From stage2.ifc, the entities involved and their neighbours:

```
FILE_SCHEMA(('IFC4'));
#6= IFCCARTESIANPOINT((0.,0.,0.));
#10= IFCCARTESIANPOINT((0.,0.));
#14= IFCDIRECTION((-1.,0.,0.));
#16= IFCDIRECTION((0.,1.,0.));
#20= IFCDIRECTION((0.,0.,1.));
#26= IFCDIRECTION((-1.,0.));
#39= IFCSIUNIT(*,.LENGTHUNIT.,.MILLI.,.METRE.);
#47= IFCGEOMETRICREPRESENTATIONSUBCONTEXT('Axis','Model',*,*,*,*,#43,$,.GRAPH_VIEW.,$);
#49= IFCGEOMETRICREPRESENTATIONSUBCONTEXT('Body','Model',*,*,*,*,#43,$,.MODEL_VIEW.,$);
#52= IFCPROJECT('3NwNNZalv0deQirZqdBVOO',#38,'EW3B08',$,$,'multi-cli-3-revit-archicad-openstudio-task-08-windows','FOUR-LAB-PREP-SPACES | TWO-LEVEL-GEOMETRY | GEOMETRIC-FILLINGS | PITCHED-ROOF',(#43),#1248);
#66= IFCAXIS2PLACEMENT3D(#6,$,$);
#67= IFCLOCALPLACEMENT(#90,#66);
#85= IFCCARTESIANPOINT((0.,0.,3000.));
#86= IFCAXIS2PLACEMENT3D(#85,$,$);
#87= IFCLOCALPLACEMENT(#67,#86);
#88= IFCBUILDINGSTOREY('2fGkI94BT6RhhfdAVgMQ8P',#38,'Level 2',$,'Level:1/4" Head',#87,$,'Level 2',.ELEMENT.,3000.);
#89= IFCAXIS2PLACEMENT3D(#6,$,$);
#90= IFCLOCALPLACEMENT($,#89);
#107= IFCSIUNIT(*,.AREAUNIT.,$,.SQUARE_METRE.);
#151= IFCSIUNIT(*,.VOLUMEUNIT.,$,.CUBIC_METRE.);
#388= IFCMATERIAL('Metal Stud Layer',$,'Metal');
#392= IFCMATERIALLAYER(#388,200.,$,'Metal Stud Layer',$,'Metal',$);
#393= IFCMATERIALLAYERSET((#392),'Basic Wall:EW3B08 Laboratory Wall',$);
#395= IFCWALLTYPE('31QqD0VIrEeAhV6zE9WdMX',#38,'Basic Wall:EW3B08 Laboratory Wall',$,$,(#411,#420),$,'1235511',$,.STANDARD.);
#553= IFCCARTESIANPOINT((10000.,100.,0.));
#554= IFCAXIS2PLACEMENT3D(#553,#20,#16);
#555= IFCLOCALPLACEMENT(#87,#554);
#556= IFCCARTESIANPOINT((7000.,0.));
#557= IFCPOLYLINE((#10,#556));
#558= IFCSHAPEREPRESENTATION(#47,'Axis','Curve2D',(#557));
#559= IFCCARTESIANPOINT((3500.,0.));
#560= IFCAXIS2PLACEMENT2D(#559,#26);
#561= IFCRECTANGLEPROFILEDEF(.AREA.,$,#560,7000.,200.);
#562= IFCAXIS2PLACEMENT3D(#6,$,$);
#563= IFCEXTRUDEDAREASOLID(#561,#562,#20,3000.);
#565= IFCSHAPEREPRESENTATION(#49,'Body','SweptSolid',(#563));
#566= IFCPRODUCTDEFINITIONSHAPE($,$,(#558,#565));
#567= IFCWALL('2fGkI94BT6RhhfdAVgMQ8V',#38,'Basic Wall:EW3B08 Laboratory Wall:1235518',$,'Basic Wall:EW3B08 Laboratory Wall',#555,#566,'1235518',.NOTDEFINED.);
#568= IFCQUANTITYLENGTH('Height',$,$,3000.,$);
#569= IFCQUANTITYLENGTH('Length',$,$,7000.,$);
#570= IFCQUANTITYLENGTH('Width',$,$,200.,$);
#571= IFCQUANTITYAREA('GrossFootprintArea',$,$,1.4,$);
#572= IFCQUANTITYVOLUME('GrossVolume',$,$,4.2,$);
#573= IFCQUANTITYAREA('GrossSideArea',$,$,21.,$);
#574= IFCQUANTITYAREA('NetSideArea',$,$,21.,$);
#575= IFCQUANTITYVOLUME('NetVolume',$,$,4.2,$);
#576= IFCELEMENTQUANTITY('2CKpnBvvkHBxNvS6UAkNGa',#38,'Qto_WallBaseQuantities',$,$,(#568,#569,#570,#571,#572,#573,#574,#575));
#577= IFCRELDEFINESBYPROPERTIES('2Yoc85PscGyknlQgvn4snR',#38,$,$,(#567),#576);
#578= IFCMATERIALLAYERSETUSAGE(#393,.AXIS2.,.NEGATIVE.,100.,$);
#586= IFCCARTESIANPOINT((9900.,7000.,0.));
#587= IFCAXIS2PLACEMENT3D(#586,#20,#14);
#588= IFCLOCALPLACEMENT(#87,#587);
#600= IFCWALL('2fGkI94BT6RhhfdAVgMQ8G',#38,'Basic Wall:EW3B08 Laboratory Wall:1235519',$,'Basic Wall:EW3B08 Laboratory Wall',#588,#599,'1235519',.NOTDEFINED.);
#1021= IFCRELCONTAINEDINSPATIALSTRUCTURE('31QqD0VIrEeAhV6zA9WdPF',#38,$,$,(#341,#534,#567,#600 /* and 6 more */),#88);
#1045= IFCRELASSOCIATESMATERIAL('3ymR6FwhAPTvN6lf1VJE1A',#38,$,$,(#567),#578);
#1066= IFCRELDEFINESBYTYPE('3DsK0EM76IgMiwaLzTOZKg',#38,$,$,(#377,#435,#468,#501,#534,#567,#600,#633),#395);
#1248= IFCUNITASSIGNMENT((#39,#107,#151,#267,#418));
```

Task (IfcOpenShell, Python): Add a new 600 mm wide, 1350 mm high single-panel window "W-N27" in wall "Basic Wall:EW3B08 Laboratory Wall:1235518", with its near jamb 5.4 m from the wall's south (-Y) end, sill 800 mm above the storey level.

```python
import numpy as np
import ifcopenshell
import ifcopenshell.api.feature
import ifcopenshell.api.geometry
import ifcopenshell.api.pset
import ifcopenshell.api.root
import ifcopenshell.api.spatial
import ifcopenshell.geom
import ifcopenshell.util.element
import ifcopenshell.util.placement
import ifcopenshell.util.representation
import ifcopenshell.util.shape
import ifcopenshell.util.unit

model = ifcopenshell.open("stage2.ifc")
unit_scale = ifcopenshell.util.unit.calculate_unit_scale(model)
area_scale = ifcopenshell.util.unit.calculate_unit_scale(model, "AREAUNIT")
volume_scale = ifcopenshell.util.unit.calculate_unit_scale(model, "VOLUMEUNIT")
settings = ifcopenshell.geom.settings()


def volume(element):
    """Net volume in cubic metres, openings subtracted."""
    shape = ifcopenshell.geom.create_shape(settings, element)
    return ifcopenshell.util.shape.get_volume(shape.geometry)


wall = model.by_id(567)
storey = ifcopenshell.util.element.get_container(wall, ifc_class="IfcBuildingStorey")
context = ifcopenshell.util.representation.get_context(model, "Model", "Body", "MODEL_VIEW")
before = volume(wall)

width, height, from_end, sill = 0.6, 1.35, 5.4, 0.8  # metres

# The wall runs along its own X axis, and the end named is its -X end.
wall_shape = ifcopenshell.geom.create_shape(settings, wall)
x, y, z = ifcopenshell.util.shape.get_vertices(wall_shape.geometry).T
start = x.min() + from_end
face, thickness = float(y.min()), float(y.max() - y.min())
wall_matrix = ifcopenshell.util.placement.get_local_placement(wall.ObjectPlacement)
level = ifcopenshell.util.placement.get_local_placement(storey.ObjectPlacement)[2, 3]


def in_wall(x, y):
    """Placement at x, y metres in the wall's axes, at sill height."""
    matrix = wall_matrix.copy()
    matrix[:, 3] = wall_matrix @ np.array([x / unit_scale, y / unit_scale, 0.0, 1.0])
    matrix[2, 3] = level + sill / unit_scale
    return matrix


# Opening: a box that overshoots both wall faces by 50 mm.
opening = ifcopenshell.api.root.create_entity(model, ifc_class="IfcOpeningElement", predefined_type="OPENING")
box = ifcopenshell.api.geometry.add_wall_representation(
    model, context=context, length=width, height=height, thickness=thickness + 0.1
)
ifcopenshell.api.geometry.assign_representation(model, product=opening, representation=box)
ifcopenshell.api.geometry.edit_object_placement(model, product=opening, matrix=in_wall(start, face - 0.05), is_si=False)
ifcopenshell.api.feature.add_feature(model, feature=opening, element=wall)

window = ifcopenshell.api.root.create_entity(model, ifc_class="IfcWindow", name="W-N27", predefined_type="WINDOW")
window.OverallWidth, window.OverallHeight = width / unit_scale, height / unit_scale
window.PartitioningType = "SINGLE_PANEL"
body = ifcopenshell.api.geometry.add_window_representation(
    model,
    context=context,
    overall_width=window.OverallWidth,
    overall_height=window.OverallHeight,
    partition_type="SINGLE_PANEL",
)
ifcopenshell.api.geometry.assign_representation(model, product=window, representation=body)
ifcopenshell.api.spatial.assign_container(model, products=[window], relating_structure=storey)
ifcopenshell.api.feature.add_filling(model, opening=opening, element=window)

# Centre the window in the wall's thickness.
ifcopenshell.api.geometry.edit_object_placement(model, product=window, matrix=in_wall(start, face), is_si=False)
window_shape = ifcopenshell.geom.create_shape(settings, window)
depth = ifcopenshell.util.shape.get_vertices(window_shape.geometry)[:, 1]
offset = face + thickness / 2 - (depth.min() + depth.max()) / 2
ifcopenshell.api.geometry.edit_object_placement(model, product=window, matrix=in_wall(start, offset), is_si=False)

after = volume(wall)

# Update the wall's stored quantities.
qto = model.by_id(ifcopenshell.util.element.get_pset(wall, "Qto_WallBaseQuantities", should_inherit=False)["id"])
ifcopenshell.api.pset.edit_qto(model, qto=qto, properties={
    "NetSideArea": after / thickness / area_scale,
    "NetVolume": after / volume_scale,
})

print(f"wall volume {before:.3f} -> {after:.3f} m3")

model.write("stage2_edited.ifc")
```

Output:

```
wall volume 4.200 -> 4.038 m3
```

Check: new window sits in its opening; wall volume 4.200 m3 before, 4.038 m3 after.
